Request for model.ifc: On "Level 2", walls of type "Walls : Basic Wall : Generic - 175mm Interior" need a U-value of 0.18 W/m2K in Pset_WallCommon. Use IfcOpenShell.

First a look at what the model holds.

```python
import ifcopenshell
import ifcopenshell.util.element

model = ifcopenshell.open("model.ifc")
print(model.schema)
storey = next(s for s in model.by_type("IfcBuildingStorey") if s.Name == "Level 2")
walls = [e for e in ifcopenshell.util.element.get_decomposition(storey) if e.is_a("IfcWall")]
seen = {}
for e in walls:
    element_type = ifcopenshell.util.element.get_type(e)
    key = (element_type.Name if element_type != e and element_type else None, ifcopenshell.util.element.get_pset(e, "Pset_WallCommon", "ThermalTransmittance"))
    seen[key] = seen.get(key, 0) + 1
for (name, value), count in sorted(seen.items(), key=str):
    print(count, "x", name, "|", value)
```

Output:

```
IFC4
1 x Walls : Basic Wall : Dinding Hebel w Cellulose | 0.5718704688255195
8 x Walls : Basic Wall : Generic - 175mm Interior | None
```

```python
import ifcopenshell
import ifcopenshell.api.pset
import ifcopenshell.util.element

model = ifcopenshell.open("model.ifc")

storey = next(s for s in model.by_type("IfcBuildingStorey") if s.Name == "Level 2")
walls = [e for e in ifcopenshell.util.element.get_decomposition(storey) if e.is_a("IfcWall")]

count = 0
for e in walls:
    element_type = ifcopenshell.util.element.get_type(e)
    if element_type in (None, e) or element_type.Name != "Walls : Basic Wall : Generic - 175mm Interior":
        continue
    # add_pset returns the element's existing set when there is one.
    pset = ifcopenshell.api.pset.add_pset(model, product=e, name="Pset_WallCommon")
    ifcopenshell.api.pset.edit_pset(model, pset=pset, properties={"ThermalTransmittance": 0.18})
    count += 1

print(count, "walls updated")

model.write("model_updated.ifc")
```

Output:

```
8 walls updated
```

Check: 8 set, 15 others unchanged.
